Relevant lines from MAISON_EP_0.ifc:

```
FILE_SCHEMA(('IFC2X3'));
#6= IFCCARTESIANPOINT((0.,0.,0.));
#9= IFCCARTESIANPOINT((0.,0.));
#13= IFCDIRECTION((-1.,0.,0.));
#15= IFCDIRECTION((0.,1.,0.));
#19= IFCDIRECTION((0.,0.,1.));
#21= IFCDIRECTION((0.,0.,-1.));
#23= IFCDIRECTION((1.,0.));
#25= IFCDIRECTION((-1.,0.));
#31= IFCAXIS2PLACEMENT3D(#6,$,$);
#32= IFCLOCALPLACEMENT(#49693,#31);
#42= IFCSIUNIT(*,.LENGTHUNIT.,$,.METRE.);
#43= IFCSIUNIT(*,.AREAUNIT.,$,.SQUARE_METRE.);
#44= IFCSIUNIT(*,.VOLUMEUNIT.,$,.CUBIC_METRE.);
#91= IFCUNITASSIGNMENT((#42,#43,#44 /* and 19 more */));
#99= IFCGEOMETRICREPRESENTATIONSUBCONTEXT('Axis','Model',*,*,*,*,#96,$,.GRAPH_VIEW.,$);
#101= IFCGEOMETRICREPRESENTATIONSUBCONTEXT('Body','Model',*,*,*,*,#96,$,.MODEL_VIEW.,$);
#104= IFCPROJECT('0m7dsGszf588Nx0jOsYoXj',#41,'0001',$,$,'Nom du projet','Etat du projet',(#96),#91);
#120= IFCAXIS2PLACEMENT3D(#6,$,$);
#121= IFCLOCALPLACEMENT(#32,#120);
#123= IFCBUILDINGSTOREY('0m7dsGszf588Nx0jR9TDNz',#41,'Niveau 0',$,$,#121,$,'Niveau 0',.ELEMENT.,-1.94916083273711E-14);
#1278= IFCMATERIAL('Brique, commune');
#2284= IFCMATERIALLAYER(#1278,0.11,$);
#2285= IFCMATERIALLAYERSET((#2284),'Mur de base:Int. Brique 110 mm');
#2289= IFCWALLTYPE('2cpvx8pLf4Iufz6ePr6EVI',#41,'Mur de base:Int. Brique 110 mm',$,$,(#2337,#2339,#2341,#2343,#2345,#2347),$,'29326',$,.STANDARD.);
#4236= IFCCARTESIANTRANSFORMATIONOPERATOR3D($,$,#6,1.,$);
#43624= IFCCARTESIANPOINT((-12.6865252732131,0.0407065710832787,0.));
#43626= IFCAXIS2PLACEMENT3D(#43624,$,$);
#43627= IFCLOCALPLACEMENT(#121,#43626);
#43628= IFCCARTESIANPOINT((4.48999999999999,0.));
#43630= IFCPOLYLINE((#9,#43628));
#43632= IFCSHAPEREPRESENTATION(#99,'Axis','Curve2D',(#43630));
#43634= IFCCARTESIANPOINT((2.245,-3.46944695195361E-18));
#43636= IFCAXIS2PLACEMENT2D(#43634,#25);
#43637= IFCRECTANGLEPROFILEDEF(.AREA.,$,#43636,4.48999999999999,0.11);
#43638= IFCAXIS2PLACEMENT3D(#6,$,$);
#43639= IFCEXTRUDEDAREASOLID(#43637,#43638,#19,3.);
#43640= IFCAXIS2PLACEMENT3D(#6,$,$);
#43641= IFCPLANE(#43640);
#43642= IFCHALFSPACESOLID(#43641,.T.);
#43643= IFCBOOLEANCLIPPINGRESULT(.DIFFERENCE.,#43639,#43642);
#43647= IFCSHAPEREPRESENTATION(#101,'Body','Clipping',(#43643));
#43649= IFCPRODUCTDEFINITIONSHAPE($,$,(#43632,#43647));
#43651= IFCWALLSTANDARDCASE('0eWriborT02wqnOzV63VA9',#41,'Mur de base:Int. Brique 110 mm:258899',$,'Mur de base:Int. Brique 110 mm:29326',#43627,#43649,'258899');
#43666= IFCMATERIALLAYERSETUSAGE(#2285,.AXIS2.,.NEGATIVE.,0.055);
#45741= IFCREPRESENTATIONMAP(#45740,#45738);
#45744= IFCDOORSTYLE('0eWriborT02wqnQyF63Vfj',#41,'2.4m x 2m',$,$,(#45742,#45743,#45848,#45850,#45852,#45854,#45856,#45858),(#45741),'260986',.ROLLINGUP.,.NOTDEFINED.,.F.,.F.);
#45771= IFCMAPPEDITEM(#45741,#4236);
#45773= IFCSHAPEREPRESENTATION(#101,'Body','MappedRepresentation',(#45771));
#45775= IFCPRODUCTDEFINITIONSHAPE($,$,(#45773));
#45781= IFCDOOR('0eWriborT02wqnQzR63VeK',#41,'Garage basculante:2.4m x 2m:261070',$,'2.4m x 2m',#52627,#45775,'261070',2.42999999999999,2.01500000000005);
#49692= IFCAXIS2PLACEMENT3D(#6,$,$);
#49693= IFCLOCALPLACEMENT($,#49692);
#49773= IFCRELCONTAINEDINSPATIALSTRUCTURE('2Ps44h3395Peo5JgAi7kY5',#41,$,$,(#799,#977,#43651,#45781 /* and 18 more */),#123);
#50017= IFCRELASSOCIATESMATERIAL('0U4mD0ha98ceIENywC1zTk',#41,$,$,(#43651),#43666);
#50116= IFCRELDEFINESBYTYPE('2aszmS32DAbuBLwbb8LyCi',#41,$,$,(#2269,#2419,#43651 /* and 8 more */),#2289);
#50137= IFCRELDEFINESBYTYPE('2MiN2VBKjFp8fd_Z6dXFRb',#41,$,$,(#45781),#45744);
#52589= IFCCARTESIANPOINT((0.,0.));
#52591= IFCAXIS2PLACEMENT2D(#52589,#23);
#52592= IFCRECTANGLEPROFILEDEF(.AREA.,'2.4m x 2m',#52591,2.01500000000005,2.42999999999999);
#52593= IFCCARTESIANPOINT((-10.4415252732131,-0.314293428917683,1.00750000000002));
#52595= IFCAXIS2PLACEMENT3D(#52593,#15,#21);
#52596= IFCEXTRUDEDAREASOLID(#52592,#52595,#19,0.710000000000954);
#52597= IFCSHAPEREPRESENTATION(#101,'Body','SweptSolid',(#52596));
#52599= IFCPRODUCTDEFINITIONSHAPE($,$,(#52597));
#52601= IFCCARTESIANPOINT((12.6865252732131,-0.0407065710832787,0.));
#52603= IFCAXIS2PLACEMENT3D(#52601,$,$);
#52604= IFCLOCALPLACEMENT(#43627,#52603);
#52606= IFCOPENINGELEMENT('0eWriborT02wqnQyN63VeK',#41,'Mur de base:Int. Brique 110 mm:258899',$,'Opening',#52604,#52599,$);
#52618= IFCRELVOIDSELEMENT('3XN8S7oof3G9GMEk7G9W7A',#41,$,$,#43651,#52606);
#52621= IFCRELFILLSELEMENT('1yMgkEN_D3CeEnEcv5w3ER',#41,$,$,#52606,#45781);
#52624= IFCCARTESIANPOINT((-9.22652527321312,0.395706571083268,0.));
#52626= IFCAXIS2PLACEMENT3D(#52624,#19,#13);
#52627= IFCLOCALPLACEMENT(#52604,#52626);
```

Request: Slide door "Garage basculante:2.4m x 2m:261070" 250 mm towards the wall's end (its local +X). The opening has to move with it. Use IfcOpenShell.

```python
import ifcopenshell
import ifcopenshell.api.geometry
import ifcopenshell.util.placement
import ifcopenshell.util.unit

model = ifcopenshell.open("MAISON_EP_0.ifc")
unit_scale = ifcopenshell.util.unit.calculate_unit_scale(model)

door = model.by_guid("0eWriborT02wqnQzR63VeK")
opening = door.FillsVoids[0].RelatingOpeningElement
wall = opening.VoidsElements[0].RelatingBuildingElement

wall_matrix = ifcopenshell.util.placement.get_local_placement(wall.ObjectPlacement)
shift = wall_matrix[:3, 0] * 0.25 / unit_scale
before = ifcopenshell.util.placement.get_local_placement(door.ObjectPlacement)[:3, 3].copy()

# The door is placed relative to its opening, so it follows when the opening moves.
matrix = ifcopenshell.util.placement.get_local_placement(opening.ObjectPlacement)
matrix[:3, 3] += shift
ifcopenshell.api.geometry.edit_object_placement(
    model, product=opening, matrix=matrix, is_si=False, should_transform_children=True
)

after = ifcopenshell.util.placement.get_local_placement(door.ObjectPlacement)[:3, 3]
print("door moved by", (after - before).round(3) + 0.0)

model.write("MAISON_EP_0_edited.ifc")
```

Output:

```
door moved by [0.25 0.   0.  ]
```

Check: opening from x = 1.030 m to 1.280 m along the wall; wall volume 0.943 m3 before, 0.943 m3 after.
